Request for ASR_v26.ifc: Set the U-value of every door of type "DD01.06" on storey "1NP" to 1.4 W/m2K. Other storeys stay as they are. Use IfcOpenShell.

First a look at what the model holds.

```python
import ifcopenshell
import ifcopenshell.util.element

model = ifcopenshell.open("ASR_v26.ifc")
print(model.schema)
storey = next(s for s in model.by_type("IfcBuildingStorey") if s.Name == "1NP")
doors = [e for e in ifcopenshell.util.element.get_decomposition(storey) if e.is_a("IfcDoor")]
seen = {}
for e in doors:
    element_type = ifcopenshell.util.element.get_type(e)
    key = (element_type.Name if element_type != e and element_type else None, ifcopenshell.util.element.get_pset(e, "Pset_DoorCommon", "ThermalTransmittance"))
    seen[key] = seen.get(key, 0) + 1
for (name, value), count in sorted(seen.items(), key=str):
    print(count, "x", name, "|", value)
```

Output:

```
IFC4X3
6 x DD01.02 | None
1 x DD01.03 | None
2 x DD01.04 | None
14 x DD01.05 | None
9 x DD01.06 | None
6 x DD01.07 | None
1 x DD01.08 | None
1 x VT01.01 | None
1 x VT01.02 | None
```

```python
import ifcopenshell
import ifcopenshell.api.pset
import ifcopenshell.util.element

model = ifcopenshell.open("ASR_v26.ifc")

storey = next(s for s in model.by_type("IfcBuildingStorey") if s.Name == "1NP")
doors = [e for e in ifcopenshell.util.element.get_decomposition(storey) if e.is_a("IfcDoor")]

count = 0
for e in doors:
    element_type = ifcopenshell.util.element.get_type(e)
    if element_type in (None, e) or element_type.Name != "DD01.06":
        continue
    # add_pset returns the element's existing set when there is one.
    pset = ifcopenshell.api.pset.add_pset(model, product=e, name="Pset_DoorCommon")
    ifcopenshell.api.pset.edit_pset(model, pset=pset, properties={"ThermalTransmittance": 1.4})
    count += 1

print(count, "doors updated")

model.write("ASR_v26_rev.ifc")
```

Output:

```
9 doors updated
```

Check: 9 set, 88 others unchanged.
